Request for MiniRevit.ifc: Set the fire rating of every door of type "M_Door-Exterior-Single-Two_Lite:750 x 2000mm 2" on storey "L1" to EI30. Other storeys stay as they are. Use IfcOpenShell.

First a look at what the model holds.

```python
import ifcopenshell
import ifcopenshell.util.element

model = ifcopenshell.open("MiniRevit.ifc")
print(model.schema)
storey = next(s for s in model.by_type("IfcBuildingStorey") if s.Name == "L1")
doors = [e for e in ifcopenshell.util.element.get_decomposition(storey) if e.is_a("IfcDoor")]
seen = {}
for e in doors:
    element_type = ifcopenshell.util.element.get_type(e)
    key = (element_type.Name if element_type != e and element_type else None, ifcopenshell.util.element.get_pset(e, "Pset_DoorCommon", "FireRating"))
    seen[key] = seen.get(key, 0) + 1
for (name, value), count in sorted(seen.items(), key=str):
    print(count, "x", name, "|", value)
```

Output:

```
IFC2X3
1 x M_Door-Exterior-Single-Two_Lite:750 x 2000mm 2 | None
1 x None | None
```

```python
import ifcopenshell
import ifcopenshell.api.pset
import ifcopenshell.util.element

model = ifcopenshell.open("MiniRevit.ifc")

storey = next(s for s in model.by_type("IfcBuildingStorey") if s.Name == "L1")
doors = [e for e in ifcopenshell.util.element.get_decomposition(storey) if e.is_a("IfcDoor")]

count = 0
for e in doors:
    element_type = ifcopenshell.util.element.get_type(e)
    if element_type in (None, e) or element_type.Name != "M_Door-Exterior-Single-Two_Lite:750 x 2000mm 2":
        continue
    # add_pset returns the element's existing set when there is one.
    pset = ifcopenshell.api.pset.add_pset(model, product=e, name="Pset_DoorCommon")
    ifcopenshell.api.pset.edit_pset(model, pset=pset, properties={"FireRating": "EI30"})
    count += 1

print(count, "doors updated")

model.write("MiniRevit_rev.ifc")
```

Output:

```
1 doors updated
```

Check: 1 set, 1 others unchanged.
